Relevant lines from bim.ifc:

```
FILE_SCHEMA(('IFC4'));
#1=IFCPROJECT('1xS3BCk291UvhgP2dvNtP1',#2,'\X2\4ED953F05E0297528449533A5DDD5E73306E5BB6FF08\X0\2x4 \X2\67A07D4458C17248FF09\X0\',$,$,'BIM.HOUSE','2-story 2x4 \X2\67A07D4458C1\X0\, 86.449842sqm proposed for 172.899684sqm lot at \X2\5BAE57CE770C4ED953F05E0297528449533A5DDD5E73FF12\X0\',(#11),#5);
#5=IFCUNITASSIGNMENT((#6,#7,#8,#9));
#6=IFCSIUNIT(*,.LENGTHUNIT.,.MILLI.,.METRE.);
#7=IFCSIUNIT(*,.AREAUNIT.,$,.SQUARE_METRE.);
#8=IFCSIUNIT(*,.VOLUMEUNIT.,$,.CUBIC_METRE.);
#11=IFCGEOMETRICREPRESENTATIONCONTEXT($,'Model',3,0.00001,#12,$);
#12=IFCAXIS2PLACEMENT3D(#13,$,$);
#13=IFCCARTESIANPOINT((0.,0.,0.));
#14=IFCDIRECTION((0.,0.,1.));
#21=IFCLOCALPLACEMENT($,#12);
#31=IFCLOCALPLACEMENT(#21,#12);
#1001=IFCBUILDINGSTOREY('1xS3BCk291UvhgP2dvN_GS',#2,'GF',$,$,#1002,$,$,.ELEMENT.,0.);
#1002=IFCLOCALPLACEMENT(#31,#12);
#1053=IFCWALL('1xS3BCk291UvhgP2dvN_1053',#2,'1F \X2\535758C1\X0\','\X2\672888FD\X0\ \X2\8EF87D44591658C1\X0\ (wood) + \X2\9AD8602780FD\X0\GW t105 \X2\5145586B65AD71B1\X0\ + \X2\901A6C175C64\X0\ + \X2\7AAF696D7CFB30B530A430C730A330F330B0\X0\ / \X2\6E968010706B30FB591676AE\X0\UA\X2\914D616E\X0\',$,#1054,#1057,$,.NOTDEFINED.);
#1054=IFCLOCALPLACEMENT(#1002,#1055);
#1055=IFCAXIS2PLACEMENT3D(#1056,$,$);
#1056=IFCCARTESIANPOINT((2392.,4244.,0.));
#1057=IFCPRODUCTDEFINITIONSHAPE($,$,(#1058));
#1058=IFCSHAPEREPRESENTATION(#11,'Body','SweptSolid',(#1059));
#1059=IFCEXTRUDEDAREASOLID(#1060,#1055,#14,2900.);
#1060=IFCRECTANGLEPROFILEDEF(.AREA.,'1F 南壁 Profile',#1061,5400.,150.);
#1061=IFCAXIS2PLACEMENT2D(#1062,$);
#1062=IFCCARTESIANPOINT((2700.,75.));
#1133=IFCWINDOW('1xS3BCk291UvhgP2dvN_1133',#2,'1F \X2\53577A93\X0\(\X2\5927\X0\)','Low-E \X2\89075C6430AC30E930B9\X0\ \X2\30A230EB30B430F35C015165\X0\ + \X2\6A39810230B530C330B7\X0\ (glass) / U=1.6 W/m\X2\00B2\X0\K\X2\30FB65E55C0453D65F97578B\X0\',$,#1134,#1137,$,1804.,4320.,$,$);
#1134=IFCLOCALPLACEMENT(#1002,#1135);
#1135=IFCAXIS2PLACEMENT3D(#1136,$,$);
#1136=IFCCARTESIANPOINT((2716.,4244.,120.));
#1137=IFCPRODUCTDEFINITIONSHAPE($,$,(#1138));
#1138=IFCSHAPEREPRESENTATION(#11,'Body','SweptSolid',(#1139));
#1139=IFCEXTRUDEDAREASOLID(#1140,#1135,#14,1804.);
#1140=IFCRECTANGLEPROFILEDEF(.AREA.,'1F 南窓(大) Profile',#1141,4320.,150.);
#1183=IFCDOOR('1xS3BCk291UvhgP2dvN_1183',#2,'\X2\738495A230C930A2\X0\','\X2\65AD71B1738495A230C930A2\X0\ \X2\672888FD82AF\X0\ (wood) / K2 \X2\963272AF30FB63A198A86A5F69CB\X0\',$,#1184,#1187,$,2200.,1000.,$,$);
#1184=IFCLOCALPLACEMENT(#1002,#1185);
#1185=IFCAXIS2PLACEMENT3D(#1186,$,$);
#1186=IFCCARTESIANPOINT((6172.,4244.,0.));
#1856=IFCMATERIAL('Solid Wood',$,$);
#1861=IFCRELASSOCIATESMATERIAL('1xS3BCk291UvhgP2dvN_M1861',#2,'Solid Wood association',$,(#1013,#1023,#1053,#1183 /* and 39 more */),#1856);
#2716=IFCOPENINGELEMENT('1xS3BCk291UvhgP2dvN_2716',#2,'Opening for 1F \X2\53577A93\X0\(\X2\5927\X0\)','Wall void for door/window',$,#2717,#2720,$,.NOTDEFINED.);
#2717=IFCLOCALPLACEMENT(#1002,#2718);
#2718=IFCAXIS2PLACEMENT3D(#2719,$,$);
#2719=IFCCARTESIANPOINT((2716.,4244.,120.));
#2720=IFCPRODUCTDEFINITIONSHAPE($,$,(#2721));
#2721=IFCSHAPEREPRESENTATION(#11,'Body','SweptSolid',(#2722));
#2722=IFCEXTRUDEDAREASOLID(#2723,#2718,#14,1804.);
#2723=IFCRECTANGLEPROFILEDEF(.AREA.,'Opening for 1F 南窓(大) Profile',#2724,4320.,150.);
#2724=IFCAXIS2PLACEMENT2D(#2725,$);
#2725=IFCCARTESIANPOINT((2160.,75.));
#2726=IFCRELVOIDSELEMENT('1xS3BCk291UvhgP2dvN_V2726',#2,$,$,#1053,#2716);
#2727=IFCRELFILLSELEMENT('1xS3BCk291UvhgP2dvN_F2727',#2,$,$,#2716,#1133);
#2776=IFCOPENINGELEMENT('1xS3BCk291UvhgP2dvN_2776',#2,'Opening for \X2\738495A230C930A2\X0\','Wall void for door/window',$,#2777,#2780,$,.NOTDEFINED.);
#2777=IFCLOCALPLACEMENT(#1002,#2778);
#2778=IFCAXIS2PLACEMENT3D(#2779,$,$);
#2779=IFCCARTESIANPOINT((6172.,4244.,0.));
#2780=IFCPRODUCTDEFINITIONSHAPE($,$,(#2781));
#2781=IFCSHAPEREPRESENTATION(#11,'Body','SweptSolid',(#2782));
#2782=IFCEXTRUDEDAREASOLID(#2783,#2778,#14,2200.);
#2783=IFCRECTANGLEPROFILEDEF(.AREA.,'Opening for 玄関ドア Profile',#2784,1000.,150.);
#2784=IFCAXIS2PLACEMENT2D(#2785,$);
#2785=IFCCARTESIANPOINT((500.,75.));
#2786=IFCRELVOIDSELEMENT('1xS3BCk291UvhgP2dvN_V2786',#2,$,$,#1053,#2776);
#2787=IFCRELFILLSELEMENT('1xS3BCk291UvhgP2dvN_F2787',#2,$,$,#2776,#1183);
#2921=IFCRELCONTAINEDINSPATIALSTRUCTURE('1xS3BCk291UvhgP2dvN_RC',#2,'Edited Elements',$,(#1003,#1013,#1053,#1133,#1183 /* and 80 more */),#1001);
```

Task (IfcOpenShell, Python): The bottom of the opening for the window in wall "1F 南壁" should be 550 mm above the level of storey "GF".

```python
import numpy as np
import ifcopenshell
import ifcopenshell.api.geometry
import ifcopenshell.geom
import ifcopenshell.util.element
import ifcopenshell.util.placement
import ifcopenshell.util.shape
import ifcopenshell.util.unit

model = ifcopenshell.open("bim.ifc")
unit_scale = ifcopenshell.util.unit.calculate_unit_scale(model)

window = model.by_guid("1xS3BCk291UvhgP2dvN_1133")
opening = window.FillsVoids[0].RelatingOpeningElement
storey = ifcopenshell.util.element.get_container(window, ifc_class="IfcBuildingStorey")
level = ifcopenshell.util.placement.get_local_placement(storey.ObjectPlacement)[2, 3]

# The opening's origin need not be at the sill, so measure its lowest point.
shape = ifcopenshell.geom.create_shape(ifcopenshell.geom.settings(), opening)
bottom = ifcopenshell.util.shape.get_shape_bottom_elevation(shape, shape.geometry) / unit_scale
dz = level + 550.0 - bottom

shift = np.array([0.0, 0.0, dz])
# The window is not placed relative to its opening, so move both.
for product in (opening, window):
    matrix = ifcopenshell.util.placement.get_local_placement(product.ObjectPlacement)
    matrix[:3, 3] += shift
    ifcopenshell.api.geometry.edit_object_placement(model, product=product, matrix=matrix, is_si=False)

print(f"moved by {dz * unit_scale:+.3f} m")

model.write("bim_v2.ifc")
```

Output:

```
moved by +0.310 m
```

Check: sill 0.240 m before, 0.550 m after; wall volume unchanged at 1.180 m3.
